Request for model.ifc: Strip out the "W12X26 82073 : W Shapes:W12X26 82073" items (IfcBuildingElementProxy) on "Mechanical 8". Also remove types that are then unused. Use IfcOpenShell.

First a look at what the model holds.

```python
import ifcopenshell
import ifcopenshell.util.element

model = ifcopenshell.open("model.ifc")
print(model.schema)
storey = next(s for s in model.by_type("IfcBuildingStorey") if s.Name == "Mechanical 8")
proxies = [e for e in ifcopenshell.util.element.get_decomposition(storey) if e.is_a("IfcBuildingElementProxy")]
seen = {}
for e in proxies:
    element_type = ifcopenshell.util.element.get_type(e)
    name = element_type.Name if element_type not in (None, e) else None
    seen[name] = seen.get(name, 0) + 1
for name, count in sorted(seen.items(), key=str):
    print(count, "x", name)
```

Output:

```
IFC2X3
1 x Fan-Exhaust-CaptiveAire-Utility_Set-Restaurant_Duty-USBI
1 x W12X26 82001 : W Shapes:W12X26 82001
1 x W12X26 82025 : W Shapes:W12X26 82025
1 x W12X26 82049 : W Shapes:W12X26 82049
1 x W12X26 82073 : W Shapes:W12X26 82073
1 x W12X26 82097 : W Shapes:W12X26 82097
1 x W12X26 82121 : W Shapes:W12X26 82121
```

```python
import ifcopenshell
import ifcopenshell.api.root
import ifcopenshell.util.element

model = ifcopenshell.open("model.ifc")

storey = next(s for s in model.by_type("IfcBuildingStorey") if s.Name == "Mechanical 8")
proxies = [e for e in ifcopenshell.util.element.get_decomposition(storey) if e.is_a("IfcBuildingElementProxy")]
targets = [e for e in proxies if (t := ifcopenshell.util.element.get_type(e)) not in (None, e) and t.Name == "W12X26 82073 : W Shapes:W12X26 82073"]
types = {ifcopenshell.util.element.get_type(e) for e in targets} - {None, *targets}

for e in targets:
    ifcopenshell.api.root.remove_product(model, product=e)
print(len(targets), "removed")

unused = [t for t in types if not ifcopenshell.util.element.get_types(t)]
for t in unused:
    ifcopenshell.api.root.remove_product(model, product=t)
print(len(unused), "unused types removed")

model.write("model_edited.ifc")
```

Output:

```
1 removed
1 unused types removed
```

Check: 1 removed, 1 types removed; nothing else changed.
